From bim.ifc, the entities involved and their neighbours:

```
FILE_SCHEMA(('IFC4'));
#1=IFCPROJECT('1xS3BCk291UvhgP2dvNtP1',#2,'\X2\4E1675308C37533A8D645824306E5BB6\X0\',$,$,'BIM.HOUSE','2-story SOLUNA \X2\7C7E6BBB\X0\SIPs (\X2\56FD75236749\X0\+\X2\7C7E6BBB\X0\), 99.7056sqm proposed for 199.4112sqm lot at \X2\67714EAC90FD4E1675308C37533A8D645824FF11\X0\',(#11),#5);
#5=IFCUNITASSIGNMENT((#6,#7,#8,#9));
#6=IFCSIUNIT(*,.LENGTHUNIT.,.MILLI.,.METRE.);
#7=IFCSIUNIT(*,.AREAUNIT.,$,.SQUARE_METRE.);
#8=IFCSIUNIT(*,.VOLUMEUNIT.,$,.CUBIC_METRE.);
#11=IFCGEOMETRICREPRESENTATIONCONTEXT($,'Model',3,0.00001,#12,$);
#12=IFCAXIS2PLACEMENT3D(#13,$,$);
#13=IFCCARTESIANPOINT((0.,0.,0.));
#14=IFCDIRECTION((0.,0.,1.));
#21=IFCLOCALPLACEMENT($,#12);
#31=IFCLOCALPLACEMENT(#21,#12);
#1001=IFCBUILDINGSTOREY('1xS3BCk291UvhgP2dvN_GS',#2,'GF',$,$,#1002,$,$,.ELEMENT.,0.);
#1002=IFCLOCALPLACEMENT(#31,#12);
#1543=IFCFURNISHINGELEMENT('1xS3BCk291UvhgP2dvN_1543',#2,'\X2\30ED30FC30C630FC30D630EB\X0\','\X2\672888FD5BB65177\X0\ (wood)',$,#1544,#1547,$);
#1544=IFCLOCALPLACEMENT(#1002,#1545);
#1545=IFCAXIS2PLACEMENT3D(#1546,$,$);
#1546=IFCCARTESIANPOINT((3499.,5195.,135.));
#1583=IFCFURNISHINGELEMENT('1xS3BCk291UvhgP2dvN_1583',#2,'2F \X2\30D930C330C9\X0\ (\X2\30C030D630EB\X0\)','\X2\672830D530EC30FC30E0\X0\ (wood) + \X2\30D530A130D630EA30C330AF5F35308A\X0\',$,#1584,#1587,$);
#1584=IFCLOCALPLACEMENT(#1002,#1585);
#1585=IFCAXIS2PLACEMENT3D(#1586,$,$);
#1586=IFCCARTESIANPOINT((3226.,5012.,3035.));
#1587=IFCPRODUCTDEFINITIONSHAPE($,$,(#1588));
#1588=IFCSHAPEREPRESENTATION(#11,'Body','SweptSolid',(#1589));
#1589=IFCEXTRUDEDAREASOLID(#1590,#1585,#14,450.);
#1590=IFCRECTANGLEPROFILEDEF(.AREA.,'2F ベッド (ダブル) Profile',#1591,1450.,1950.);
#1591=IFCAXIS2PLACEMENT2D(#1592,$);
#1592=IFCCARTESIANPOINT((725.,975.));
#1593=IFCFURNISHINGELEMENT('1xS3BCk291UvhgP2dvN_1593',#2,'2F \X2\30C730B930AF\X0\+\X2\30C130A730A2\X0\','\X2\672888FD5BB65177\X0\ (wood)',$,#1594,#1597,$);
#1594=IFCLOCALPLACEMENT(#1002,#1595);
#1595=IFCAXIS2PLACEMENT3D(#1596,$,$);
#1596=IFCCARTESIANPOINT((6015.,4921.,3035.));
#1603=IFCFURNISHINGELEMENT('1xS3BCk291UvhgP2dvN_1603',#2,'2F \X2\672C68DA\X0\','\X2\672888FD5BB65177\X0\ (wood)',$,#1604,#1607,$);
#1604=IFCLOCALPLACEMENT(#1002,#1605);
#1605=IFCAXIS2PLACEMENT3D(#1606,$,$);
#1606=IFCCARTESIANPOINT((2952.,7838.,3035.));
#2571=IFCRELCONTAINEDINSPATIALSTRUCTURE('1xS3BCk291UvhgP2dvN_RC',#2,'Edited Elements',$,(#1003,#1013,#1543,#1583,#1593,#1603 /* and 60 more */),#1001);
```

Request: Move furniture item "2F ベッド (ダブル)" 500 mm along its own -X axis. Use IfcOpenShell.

```python
import ifcopenshell
import ifcopenshell.api.geometry
import ifcopenshell.util.placement

model = ifcopenshell.open("bim.ifc")

item = model.by_id(1583)
matrix = ifcopenshell.util.placement.get_local_placement(item.ObjectPlacement)
matrix[:3, 3] -= matrix[:3, 0] * 500.0
ifcopenshell.api.geometry.edit_object_placement(model, product=item, matrix=matrix, is_si=False)

print(ifcopenshell.util.placement.get_local_placement(item.ObjectPlacement).round(3) + 0.0)

model.write("bim_updated.ifc")
```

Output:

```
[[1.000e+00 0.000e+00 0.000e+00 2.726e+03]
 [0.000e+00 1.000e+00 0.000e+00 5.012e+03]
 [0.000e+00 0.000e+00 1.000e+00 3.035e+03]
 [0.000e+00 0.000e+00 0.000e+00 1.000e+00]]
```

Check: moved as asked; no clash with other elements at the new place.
